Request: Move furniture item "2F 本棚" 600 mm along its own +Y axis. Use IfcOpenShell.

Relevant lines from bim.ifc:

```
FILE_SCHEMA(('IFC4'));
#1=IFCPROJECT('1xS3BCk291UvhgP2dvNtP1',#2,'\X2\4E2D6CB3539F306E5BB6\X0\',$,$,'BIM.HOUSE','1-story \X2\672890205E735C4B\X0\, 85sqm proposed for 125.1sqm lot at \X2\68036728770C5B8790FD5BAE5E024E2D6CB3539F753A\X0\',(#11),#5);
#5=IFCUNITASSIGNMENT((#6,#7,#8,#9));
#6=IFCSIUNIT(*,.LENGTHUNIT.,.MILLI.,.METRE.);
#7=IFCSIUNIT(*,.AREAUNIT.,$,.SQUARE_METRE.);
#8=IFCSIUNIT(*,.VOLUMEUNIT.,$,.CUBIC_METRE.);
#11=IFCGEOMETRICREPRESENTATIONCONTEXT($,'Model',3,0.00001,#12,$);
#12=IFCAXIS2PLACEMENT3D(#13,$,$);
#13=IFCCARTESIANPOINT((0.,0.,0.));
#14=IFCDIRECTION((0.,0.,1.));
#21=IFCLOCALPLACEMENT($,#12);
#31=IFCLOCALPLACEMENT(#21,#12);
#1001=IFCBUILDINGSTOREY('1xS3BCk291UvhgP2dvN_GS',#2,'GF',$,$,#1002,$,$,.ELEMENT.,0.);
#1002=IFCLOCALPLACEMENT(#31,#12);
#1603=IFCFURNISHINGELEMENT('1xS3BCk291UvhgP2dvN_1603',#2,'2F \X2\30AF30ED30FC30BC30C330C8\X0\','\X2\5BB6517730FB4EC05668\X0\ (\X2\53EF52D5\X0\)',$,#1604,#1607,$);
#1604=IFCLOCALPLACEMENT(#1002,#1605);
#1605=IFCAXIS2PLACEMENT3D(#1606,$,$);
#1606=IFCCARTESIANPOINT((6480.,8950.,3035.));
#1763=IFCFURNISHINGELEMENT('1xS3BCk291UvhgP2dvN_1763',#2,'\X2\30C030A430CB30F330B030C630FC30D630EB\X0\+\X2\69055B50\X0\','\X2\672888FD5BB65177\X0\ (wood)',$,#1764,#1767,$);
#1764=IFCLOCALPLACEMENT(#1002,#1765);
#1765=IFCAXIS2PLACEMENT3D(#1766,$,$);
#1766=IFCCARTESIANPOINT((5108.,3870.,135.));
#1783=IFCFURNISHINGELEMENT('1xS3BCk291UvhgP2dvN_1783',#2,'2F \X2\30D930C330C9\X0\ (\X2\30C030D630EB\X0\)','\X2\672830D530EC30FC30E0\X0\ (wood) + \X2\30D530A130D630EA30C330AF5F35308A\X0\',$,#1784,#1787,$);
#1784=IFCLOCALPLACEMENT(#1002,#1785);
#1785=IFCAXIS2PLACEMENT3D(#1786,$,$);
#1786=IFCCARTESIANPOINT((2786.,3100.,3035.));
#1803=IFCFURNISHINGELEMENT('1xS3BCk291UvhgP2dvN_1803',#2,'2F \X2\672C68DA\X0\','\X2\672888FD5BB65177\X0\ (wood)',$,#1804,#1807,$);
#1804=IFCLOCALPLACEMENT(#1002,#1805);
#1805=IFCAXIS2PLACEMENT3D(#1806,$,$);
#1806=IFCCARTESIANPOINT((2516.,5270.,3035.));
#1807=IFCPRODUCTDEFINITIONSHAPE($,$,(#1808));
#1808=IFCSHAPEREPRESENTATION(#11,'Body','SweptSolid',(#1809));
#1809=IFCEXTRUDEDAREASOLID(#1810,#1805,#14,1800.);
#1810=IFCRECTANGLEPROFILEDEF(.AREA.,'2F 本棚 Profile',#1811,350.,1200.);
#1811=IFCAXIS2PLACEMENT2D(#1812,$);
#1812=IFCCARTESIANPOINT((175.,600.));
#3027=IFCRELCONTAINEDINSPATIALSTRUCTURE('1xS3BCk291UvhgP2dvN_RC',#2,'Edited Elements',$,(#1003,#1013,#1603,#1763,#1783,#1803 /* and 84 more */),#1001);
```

```python
import ifcopenshell
import ifcopenshell.api.geometry
import ifcopenshell.util.placement

model = ifcopenshell.open("bim.ifc")

item = model.by_guid("1xS3BCk291UvhgP2dvN_1803")
matrix = ifcopenshell.util.placement.get_local_placement(item.ObjectPlacement)
matrix[:3, 3] += matrix[:3, 1] * 600.0
ifcopenshell.api.geometry.edit_object_placement(model, product=item, matrix=matrix, is_si=False)

print(ifcopenshell.util.placement.get_local_placement(item.ObjectPlacement).round(3) + 0.0)

model.write("bim-out.ifc")
```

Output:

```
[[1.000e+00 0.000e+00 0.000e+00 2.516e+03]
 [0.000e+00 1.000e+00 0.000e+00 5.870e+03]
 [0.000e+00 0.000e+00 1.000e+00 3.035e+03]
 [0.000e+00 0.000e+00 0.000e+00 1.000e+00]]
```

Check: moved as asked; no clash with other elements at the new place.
